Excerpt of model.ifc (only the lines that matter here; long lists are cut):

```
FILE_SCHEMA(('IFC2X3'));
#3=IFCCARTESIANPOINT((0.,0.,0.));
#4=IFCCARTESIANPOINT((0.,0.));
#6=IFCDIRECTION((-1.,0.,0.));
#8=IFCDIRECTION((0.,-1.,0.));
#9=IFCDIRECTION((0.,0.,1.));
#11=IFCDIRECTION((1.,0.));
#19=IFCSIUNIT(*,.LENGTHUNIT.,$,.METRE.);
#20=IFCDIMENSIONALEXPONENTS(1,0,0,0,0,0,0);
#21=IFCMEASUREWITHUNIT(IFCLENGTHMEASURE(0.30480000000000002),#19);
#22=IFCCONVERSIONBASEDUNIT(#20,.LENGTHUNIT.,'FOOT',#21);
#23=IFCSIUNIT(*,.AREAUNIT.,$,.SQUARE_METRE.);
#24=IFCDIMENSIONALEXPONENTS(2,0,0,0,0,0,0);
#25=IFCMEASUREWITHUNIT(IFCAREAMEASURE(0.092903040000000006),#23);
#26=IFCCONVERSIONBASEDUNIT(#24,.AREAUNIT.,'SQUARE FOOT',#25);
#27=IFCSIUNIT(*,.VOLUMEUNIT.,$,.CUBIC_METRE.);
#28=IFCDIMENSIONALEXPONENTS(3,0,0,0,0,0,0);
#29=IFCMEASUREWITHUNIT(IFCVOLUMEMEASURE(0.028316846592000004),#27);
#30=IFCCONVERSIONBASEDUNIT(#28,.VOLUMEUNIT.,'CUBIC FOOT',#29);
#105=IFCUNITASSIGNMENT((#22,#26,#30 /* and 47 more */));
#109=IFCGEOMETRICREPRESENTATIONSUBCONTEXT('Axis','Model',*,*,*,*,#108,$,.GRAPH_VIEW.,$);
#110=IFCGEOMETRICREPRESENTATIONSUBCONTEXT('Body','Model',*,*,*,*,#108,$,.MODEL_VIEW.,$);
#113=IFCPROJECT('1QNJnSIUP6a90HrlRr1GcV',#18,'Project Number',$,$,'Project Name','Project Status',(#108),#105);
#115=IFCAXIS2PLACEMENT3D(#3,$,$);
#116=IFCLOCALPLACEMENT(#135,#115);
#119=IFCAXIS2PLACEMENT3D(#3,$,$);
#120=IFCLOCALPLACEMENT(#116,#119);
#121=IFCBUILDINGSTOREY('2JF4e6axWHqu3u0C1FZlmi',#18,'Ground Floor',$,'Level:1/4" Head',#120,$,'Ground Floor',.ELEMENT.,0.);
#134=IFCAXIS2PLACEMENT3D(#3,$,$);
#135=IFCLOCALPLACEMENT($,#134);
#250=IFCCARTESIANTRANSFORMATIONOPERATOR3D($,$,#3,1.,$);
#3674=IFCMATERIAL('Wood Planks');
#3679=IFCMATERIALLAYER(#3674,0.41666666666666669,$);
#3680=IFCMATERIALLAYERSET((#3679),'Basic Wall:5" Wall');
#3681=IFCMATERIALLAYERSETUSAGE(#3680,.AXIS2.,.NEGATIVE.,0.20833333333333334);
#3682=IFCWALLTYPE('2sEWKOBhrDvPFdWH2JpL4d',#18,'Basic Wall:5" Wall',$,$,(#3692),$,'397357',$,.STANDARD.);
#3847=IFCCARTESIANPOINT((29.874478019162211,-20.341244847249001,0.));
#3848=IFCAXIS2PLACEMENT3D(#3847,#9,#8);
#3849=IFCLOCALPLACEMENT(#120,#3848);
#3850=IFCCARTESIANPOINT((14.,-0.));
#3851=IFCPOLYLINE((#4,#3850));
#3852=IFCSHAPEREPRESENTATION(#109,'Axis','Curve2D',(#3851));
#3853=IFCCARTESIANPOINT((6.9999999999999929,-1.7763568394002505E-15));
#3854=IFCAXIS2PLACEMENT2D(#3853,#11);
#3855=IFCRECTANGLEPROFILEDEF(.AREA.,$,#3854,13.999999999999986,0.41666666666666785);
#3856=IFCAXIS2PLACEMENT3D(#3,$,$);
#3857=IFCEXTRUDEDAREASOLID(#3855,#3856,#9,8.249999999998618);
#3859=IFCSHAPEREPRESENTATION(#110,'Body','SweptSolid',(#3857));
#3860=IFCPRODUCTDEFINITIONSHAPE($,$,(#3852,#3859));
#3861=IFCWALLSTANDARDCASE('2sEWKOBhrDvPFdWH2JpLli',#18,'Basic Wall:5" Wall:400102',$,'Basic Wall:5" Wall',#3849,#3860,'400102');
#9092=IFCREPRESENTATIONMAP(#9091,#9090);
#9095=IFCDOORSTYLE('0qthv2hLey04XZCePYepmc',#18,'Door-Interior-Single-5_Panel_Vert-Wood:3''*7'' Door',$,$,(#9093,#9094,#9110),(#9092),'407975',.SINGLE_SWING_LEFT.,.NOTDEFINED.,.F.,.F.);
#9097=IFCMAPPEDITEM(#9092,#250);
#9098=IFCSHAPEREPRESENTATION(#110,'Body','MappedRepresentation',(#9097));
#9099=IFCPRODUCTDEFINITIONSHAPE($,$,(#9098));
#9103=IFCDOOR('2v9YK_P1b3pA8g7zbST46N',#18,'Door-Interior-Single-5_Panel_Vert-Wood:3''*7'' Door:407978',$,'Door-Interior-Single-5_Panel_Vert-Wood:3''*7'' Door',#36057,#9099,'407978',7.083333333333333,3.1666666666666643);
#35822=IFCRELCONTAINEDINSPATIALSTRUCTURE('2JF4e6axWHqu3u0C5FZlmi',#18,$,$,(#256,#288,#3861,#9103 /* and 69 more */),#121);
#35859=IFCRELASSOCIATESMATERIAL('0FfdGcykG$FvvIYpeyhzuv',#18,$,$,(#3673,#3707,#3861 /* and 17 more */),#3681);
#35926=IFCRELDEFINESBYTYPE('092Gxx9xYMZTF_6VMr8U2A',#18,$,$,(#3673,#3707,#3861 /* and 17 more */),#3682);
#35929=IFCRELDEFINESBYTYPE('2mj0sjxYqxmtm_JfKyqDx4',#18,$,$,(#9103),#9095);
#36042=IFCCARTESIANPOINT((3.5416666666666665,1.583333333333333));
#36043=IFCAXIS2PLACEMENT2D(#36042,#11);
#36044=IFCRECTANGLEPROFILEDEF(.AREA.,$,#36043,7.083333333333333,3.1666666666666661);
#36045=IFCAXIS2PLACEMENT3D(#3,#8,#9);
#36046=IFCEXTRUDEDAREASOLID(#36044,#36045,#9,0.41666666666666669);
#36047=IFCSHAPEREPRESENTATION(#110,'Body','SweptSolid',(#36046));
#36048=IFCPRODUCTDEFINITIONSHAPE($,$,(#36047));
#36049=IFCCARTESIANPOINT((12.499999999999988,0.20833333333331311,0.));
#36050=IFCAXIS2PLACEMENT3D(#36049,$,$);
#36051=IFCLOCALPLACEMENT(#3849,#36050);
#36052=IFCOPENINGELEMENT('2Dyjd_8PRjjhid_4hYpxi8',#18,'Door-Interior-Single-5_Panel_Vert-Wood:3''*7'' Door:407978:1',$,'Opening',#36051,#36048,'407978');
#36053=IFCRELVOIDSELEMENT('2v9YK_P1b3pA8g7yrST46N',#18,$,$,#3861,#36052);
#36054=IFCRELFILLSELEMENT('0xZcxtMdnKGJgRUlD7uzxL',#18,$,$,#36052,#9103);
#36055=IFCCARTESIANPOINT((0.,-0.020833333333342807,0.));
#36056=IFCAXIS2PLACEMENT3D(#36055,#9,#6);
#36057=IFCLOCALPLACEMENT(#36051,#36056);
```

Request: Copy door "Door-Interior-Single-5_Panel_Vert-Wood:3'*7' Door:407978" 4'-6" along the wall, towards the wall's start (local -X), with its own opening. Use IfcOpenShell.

```python
import ifcopenshell
import ifcopenshell.api.feature
import ifcopenshell.api.geometry
import ifcopenshell.api.root
import ifcopenshell.geom
import ifcopenshell.util.element
import ifcopenshell.util.placement
import ifcopenshell.util.shape
import ifcopenshell.util.unit

model = ifcopenshell.open("model.ifc")
unit_scale = ifcopenshell.util.unit.calculate_unit_scale(model)
settings = ifcopenshell.geom.settings()


def volume(element):
    """Net volume in cubic metres, openings subtracted."""
    shape = ifcopenshell.geom.create_shape(settings, element)
    return ifcopenshell.util.shape.get_volume(shape.geometry)


def reuse_history(source, copy):
    """copy_class also copies each property set's owner history, people and application; keep the originals."""
    for rel in copy.IsDefinedBy:
        if rel.is_a("IfcRelDefinesByProperties") and (history := rel.RelatingPropertyDefinition.OwnerHistory):
            rel.RelatingPropertyDefinition.OwnerHistory = source.OwnerHistory
            ifcopenshell.util.element.remove_deep2(model, history)


door = model.by_guid("2v9YK_P1b3pA8g7zbST46N")
opening = door.FillsVoids[0].RelatingOpeningElement
wall = opening.VoidsElements[0].RelatingBuildingElement
before = volume(wall)
shift = ifcopenshell.util.placement.get_local_placement(wall.ObjectPlacement)[:3, 0] * -54 * 0.0254 / unit_scale

# copy_class copies the void relationship, type, container and properties, but no geometry.
new_opening = ifcopenshell.api.root.copy_class(model, product=opening)
new_opening.Representation = ifcopenshell.util.element.copy_deep(
    model, opening.Representation, exclude=["IfcGeometricRepresentationContext", "IfcRepresentationMap"]
)
new_opening.Name = "Door-Interior-Single-5_Panel_Vert-Wood:3'*7' Door"
new_opening.Tag = None
new_door = ifcopenshell.api.root.copy_class(model, product=door)
new_door.Representation = ifcopenshell.util.element.copy_deep(
    model, door.Representation, exclude=["IfcGeometricRepresentationContext", "IfcRepresentationMap"]
)
new_door.Name = "Door-Interior-Single-5_Panel_Vert-Wood:3'*7' Door"
new_door.Tag = None
reuse_history(door, new_door)
fills = ifcopenshell.api.feature.add_filling(model, opening=new_opening, element=new_door)
fills.OwnerHistory = new_door.OwnerHistory  # required in IFC2X3

for old, new in ((opening, new_opening), (door, new_door)):
    matrix = ifcopenshell.util.placement.get_local_placement(old.ObjectPlacement)
    matrix[:3, 3] += shift
    ifcopenshell.api.geometry.edit_object_placement(model, product=new, matrix=matrix, is_si=False)

after = volume(wall)

print(f"wall volume {before:.3f} -> {after:.3f} m3")

model.write("model_edited.ifc")
```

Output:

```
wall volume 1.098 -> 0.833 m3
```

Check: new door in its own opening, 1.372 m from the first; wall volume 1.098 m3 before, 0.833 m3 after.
